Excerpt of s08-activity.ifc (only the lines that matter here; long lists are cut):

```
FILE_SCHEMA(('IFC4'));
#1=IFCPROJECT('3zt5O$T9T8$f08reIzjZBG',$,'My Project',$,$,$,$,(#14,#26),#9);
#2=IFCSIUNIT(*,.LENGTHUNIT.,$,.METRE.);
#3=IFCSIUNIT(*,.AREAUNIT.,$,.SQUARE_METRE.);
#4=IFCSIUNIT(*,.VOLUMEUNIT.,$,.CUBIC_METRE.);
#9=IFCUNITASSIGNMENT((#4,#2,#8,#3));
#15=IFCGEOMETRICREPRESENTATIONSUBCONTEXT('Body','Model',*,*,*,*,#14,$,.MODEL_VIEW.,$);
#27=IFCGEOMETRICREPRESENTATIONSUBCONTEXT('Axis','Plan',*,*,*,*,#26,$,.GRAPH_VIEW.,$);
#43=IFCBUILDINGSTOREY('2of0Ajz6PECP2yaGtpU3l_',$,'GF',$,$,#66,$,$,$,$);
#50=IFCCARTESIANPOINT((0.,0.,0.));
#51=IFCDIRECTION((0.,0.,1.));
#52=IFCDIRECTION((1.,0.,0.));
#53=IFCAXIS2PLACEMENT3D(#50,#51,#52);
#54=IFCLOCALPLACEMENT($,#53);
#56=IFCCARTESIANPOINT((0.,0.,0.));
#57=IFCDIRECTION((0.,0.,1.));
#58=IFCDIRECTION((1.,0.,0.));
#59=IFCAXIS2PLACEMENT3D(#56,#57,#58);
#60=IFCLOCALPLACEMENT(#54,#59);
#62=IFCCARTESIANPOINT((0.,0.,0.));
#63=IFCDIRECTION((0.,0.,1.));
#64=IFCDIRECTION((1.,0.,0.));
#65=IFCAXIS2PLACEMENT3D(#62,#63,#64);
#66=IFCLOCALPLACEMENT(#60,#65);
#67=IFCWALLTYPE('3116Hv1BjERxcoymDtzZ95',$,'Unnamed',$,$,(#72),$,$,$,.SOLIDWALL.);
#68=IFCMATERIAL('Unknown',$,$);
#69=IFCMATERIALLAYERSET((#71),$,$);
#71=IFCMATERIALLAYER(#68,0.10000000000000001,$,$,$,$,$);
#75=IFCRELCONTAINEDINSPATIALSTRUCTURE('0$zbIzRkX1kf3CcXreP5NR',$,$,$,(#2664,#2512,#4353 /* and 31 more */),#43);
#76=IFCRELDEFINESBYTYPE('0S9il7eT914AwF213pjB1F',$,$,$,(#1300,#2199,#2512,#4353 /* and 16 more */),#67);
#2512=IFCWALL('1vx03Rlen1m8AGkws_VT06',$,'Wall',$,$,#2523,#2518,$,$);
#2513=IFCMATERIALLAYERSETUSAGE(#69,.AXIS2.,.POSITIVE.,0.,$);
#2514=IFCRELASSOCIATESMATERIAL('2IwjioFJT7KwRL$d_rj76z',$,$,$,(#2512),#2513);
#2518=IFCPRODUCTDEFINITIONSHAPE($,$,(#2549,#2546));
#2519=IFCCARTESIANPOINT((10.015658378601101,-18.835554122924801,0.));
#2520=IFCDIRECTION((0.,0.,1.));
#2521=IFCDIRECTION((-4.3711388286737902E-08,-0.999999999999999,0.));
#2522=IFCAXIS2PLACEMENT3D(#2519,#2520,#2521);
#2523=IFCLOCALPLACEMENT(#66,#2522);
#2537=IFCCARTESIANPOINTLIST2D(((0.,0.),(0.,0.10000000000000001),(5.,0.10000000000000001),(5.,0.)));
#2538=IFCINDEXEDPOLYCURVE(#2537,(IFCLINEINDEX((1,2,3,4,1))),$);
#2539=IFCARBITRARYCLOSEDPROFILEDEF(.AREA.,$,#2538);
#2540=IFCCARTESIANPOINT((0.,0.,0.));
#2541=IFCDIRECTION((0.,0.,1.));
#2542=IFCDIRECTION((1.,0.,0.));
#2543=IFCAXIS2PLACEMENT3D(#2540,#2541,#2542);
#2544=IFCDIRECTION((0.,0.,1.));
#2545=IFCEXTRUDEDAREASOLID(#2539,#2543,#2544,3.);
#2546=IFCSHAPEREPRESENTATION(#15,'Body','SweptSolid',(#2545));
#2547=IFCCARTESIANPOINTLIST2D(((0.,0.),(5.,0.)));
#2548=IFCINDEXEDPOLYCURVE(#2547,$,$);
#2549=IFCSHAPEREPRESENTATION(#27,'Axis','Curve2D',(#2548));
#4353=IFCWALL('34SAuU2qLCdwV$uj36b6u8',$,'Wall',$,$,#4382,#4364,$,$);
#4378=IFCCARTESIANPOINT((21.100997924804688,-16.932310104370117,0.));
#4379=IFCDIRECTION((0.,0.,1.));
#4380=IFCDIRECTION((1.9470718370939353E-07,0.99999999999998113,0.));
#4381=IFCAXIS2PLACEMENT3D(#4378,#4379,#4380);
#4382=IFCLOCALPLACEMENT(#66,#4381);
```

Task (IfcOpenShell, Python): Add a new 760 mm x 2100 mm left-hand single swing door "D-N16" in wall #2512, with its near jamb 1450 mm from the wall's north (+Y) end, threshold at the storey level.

```python
import numpy as np
import ifcopenshell
import ifcopenshell.api.feature
import ifcopenshell.api.geometry
import ifcopenshell.api.root
import ifcopenshell.api.spatial
import ifcopenshell.geom
import ifcopenshell.util.element
import ifcopenshell.util.placement
import ifcopenshell.util.representation
import ifcopenshell.util.shape
import ifcopenshell.util.unit

model = ifcopenshell.open("s08-activity.ifc")
unit_scale = ifcopenshell.util.unit.calculate_unit_scale(model)
settings = ifcopenshell.geom.settings()


def volume(element):
    """Net volume in cubic metres, openings subtracted."""
    shape = ifcopenshell.geom.create_shape(settings, element)
    return ifcopenshell.util.shape.get_volume(shape.geometry)


wall = model.by_guid("1vx03Rlen1m8AGkws_VT06")
storey = ifcopenshell.util.element.get_container(wall, ifc_class="IfcBuildingStorey")
context = ifcopenshell.util.representation.get_context(model, "Model", "Body", "MODEL_VIEW")
before = volume(wall)

width, height, from_end, sill = 0.76, 2.1, 1.45, 0.0  # metres

# The wall runs along its own X axis, and the end named is its -X end.
wall_shape = ifcopenshell.geom.create_shape(settings, wall)
x, y, z = ifcopenshell.util.shape.get_vertices(wall_shape.geometry).T
start = x.min() + from_end
face, thickness = float(y.min()), float(y.max() - y.min())
wall_matrix = ifcopenshell.util.placement.get_local_placement(wall.ObjectPlacement)
level = ifcopenshell.util.placement.get_local_placement(storey.ObjectPlacement)[2, 3]


def in_wall(x, y):
    """Placement at x, y metres in the wall's axes, at sill height."""
    matrix = wall_matrix.copy()
    matrix[:, 3] = wall_matrix @ np.array([x / unit_scale, y / unit_scale, 0.0, 1.0])
    matrix[2, 3] = level + sill / unit_scale
    return matrix


# Opening: a box that overshoots both wall faces by 50 mm.
opening = ifcopenshell.api.root.create_entity(model, ifc_class="IfcOpeningElement", predefined_type="OPENING")
box = ifcopenshell.api.geometry.add_wall_representation(
    model, context=context, length=width, height=height, thickness=thickness + 0.1
)
ifcopenshell.api.geometry.assign_representation(model, product=opening, representation=box)
ifcopenshell.api.geometry.edit_object_placement(model, product=opening, matrix=in_wall(start, face - 0.05), is_si=False)
ifcopenshell.api.feature.add_feature(model, feature=opening, element=wall)

door = ifcopenshell.api.root.create_entity(model, ifc_class="IfcDoor", name="D-N16", predefined_type="DOOR")
door.OverallWidth, door.OverallHeight = width / unit_scale, height / unit_scale
door.OperationType = "SINGLE_SWING_LEFT"
body = ifcopenshell.api.geometry.add_door_representation(
    model,
    context=context,
    overall_width=door.OverallWidth,
    overall_height=door.OverallHeight,
    operation_type="SINGLE_SWING_LEFT",
    lining_properties={"LiningDepth": thickness / unit_scale, "ThresholdDepth": thickness / unit_scale},
)
ifcopenshell.api.geometry.assign_representation(model, product=door, representation=body)
ifcopenshell.api.spatial.assign_container(model, products=[door], relating_structure=storey)
ifcopenshell.api.feature.add_filling(model, opening=opening, element=door)

# The lining spans the wall, so the door starts at the wall face.
ifcopenshell.api.geometry.edit_object_placement(model, product=door, matrix=in_wall(start, face), is_si=False)

after = volume(wall)

print(f"wall volume {before:.3f} -> {after:.3f} m3")

model.write("s08-activity-out.ifc")
```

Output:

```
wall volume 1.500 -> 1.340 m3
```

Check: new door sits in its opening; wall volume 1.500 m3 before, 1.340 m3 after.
